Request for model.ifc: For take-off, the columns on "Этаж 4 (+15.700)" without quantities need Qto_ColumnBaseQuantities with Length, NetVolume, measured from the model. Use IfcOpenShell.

First a look at what the model holds.

```python
import ifcopenshell
import ifcopenshell.util.element
import ifcopenshell.util.unit

model = ifcopenshell.open("model.ifc")
print(model.schema)
for unit_type in ("LENGTHUNIT", "AREAUNIT", "VOLUMEUNIT"):
    print(unit_type, ifcopenshell.util.unit.calculate_unit_scale(model, unit_type))
storey = next(s for s in model.by_type("IfcBuildingStorey") if s.Name == "Этаж 4 (+15.700)")
columns = [e for e in ifcopenshell.util.element.get_decomposition(storey) if e.is_a("IfcColumn")]
for e in sorted(columns, key=lambda e: e.id()):
    print(e.id(), e.is_a(), e.Name, list(ifcopenshell.util.element.get_psets(e, qtos_only=True)), sep=" | ")
```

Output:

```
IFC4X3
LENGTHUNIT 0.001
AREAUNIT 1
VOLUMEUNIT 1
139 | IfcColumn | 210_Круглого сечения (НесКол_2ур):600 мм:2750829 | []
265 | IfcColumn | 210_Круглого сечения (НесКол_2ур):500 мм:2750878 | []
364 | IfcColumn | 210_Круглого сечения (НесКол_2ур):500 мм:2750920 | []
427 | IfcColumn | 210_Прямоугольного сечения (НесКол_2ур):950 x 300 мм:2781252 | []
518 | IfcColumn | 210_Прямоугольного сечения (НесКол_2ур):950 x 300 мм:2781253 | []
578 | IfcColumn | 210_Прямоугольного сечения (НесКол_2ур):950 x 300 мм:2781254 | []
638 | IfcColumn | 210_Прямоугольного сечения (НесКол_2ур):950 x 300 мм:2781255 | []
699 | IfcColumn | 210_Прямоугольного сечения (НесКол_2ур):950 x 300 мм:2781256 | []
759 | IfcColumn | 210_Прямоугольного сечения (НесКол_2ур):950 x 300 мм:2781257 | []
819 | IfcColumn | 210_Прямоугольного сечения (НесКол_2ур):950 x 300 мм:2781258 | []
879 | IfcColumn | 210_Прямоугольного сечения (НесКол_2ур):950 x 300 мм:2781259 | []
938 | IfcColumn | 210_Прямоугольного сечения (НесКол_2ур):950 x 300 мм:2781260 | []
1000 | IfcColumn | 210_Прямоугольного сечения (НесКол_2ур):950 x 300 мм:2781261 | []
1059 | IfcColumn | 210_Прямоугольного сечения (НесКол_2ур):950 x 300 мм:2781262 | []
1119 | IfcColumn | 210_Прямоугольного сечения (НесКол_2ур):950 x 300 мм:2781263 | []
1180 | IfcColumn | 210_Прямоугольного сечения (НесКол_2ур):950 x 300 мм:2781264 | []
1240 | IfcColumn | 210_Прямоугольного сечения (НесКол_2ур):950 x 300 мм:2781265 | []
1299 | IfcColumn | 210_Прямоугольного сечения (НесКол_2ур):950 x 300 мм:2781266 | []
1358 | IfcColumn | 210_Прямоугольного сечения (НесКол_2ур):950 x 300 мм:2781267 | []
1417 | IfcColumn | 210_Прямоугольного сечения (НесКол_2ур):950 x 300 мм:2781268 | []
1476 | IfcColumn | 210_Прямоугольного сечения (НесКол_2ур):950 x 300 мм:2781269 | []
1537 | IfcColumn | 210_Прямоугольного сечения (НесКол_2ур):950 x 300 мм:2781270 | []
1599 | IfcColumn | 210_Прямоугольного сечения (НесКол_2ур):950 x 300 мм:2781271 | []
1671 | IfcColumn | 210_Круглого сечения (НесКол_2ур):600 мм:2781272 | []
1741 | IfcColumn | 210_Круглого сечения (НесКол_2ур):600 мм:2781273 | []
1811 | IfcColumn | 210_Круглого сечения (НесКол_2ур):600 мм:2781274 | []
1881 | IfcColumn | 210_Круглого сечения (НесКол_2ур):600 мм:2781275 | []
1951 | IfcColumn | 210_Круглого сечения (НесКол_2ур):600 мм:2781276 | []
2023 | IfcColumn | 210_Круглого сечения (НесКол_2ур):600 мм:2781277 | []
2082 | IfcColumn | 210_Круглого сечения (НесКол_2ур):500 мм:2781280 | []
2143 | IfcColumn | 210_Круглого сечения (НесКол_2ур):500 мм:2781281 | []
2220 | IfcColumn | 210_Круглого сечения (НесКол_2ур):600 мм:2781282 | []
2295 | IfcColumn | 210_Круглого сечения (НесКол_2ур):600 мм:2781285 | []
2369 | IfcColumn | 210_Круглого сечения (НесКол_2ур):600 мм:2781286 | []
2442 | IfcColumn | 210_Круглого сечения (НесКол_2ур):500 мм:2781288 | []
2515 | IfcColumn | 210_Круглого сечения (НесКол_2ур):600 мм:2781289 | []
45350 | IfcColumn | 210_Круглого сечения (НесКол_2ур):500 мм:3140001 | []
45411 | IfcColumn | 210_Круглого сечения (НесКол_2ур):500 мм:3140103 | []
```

```python
import ifcopenshell
import ifcopenshell.api.pset
import ifcopenshell.geom
import ifcopenshell.util.element
import ifcopenshell.util.shape
import ifcopenshell.util.unit

model = ifcopenshell.open("model.ifc")
unit_scale = ifcopenshell.util.unit.calculate_unit_scale(model)
volume_scale = ifcopenshell.util.unit.calculate_unit_scale(model, "VOLUMEUNIT")
settings = ifcopenshell.geom.settings()

storey = next(s for s in model.by_type("IfcBuildingStorey") if s.Name == "Этаж 4 (+15.700)")
columns = [e for e in ifcopenshell.util.element.get_decomposition(storey) if e.is_a("IfcColumn")]

for e in sorted(columns, key=lambda e: e.id()):
    if ifcopenshell.util.element.get_psets(e, qtos_only=True, should_inherit=False):
        continue
    # Geometry comes back in metres, in the element's own axes.
    shape = ifcopenshell.geom.create_shape(settings, e)
    values = {
        "Length": ifcopenshell.util.shape.get_z(shape.geometry) / unit_scale,
        "NetVolume": ifcopenshell.util.shape.get_volume(shape.geometry) / volume_scale,
    }
    qto = ifcopenshell.api.pset.add_qto(model, product=e, name="Qto_ColumnBaseQuantities")
    ifcopenshell.api.pset.edit_qto(model, qto=qto, properties=values)
    print(e.id(), {k: round(v, 3) for k, v in values.items()})

model.write("model-out.ifc")
```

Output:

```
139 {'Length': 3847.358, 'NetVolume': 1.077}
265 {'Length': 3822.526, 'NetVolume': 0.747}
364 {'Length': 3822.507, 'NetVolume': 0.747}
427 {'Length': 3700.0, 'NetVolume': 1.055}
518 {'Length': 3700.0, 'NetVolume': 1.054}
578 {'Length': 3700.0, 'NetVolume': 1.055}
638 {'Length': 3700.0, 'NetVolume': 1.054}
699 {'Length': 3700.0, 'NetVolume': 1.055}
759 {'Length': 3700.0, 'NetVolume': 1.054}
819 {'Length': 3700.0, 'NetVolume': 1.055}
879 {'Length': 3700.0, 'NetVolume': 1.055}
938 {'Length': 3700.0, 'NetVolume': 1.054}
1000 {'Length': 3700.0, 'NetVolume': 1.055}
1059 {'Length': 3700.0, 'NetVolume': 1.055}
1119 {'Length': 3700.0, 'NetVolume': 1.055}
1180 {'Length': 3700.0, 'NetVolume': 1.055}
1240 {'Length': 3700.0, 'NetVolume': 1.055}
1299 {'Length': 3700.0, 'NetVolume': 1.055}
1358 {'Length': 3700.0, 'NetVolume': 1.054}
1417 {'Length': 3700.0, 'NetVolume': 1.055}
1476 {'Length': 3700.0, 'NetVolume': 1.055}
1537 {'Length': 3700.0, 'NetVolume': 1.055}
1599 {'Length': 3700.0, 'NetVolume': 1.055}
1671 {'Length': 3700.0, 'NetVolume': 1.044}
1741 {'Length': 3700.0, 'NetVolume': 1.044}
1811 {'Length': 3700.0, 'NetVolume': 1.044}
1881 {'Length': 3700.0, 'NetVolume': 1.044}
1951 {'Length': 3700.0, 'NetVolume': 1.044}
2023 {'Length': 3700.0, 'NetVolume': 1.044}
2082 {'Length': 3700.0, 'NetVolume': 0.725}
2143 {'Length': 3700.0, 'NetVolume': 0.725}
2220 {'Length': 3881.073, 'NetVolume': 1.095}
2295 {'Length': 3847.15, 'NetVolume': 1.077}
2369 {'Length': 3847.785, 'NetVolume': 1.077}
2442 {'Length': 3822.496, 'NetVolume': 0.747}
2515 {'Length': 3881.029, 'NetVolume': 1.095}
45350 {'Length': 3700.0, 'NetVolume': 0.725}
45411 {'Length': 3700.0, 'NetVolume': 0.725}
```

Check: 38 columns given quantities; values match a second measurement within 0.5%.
